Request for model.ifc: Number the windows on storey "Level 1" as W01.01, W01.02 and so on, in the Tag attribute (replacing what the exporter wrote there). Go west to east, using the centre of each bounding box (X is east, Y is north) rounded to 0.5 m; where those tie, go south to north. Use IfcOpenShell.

First a look at what the model holds.

```python
import ifcopenshell
import ifcopenshell.util.element
import ifcopenshell.util.placement

model = ifcopenshell.open("model.ifc")
print(model.schema)
storey = next(s for s in model.by_type("IfcBuildingStorey") if s.Name == "Level 1")
windows = [e for e in ifcopenshell.util.element.get_decomposition(storey) if e.is_a("IfcWindow")]
for e in sorted(windows, key=lambda e: e.id()):
    origin = ifcopenshell.util.placement.get_local_placement(e.ObjectPlacement)[:3, 3]
    print(e.id(), e.Tag, e.Name, origin.round(2) + 0.0, sep=" | ")
```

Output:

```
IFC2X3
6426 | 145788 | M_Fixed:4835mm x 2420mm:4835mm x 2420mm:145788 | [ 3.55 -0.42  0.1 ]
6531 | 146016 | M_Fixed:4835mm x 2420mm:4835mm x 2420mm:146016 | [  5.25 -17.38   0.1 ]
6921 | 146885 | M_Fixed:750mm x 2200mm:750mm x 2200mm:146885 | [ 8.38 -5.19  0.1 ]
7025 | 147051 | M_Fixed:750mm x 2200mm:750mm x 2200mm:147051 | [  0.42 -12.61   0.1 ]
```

```python
import ifcopenshell
import ifcopenshell.geom
import ifcopenshell.util.element
import ifcopenshell.util.shape

model = ifcopenshell.open("model.ifc")
settings = ifcopenshell.geom.settings()
settings.set("use-world-coords", True)


def centre(element):
    shape = ifcopenshell.geom.create_shape(settings, element)
    return ifcopenshell.util.shape.get_bbox_centroid(shape.geometry)


storey = next(s for s in model.by_type("IfcBuildingStorey") if s.Name == "Level 1")
windows = [e for e in ifcopenshell.util.element.get_decomposition(storey) if e.is_a("IfcWindow")]

# Insertion points can sit at a corner or the storey origin, so sort by the geometry (in metres).
centres = {e: centre(e) for e in windows}
windows.sort(key=lambda e: (round(centres[e][0] / 0.5), centres[e][1]))

for i, e in enumerate(windows, start=1):
    number = f"W01.{i:02d}"
    e.Tag = number
    print(e.id(), number)

model.write("model_edited.ifc")
```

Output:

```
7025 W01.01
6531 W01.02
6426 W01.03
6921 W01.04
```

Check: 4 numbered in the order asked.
